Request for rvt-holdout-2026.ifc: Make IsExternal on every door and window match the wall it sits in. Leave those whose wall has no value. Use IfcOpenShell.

First a look at what the model holds.

```python
import ifcopenshell
import ifcopenshell.util.element

model = ifcopenshell.open("rvt-holdout-2026.ifc")
print(model.schema)
seen = {}
for e in model.by_type("IfcDoor") + model.by_type("IfcWindow"):
    if not e.FillsVoids:
        continue
    host = e.FillsVoids[0].RelatingOpeningElement.VoidsElements[0].RelatingBuildingElement
    own = ifcopenshell.util.element.get_pset(e, f"Pset_{e.is_a()[3:].removesuffix('StandardCase')}Common", "IsExternal")
    wall = ifcopenshell.util.element.get_pset(host, "Pset_WallCommon", "IsExternal")
    seen[e.is_a(), own, wall] = seen.get((e.is_a(), own, wall), 0) + 1
for (cls, own, wall), count in sorted(seen.items(), key=str):
    print(count, cls, "IsExternal:", own, "| host wall:", wall)
```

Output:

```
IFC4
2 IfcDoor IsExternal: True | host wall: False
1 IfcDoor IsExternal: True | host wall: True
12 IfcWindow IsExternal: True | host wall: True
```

```python
import ifcopenshell
import ifcopenshell.api.pset
import ifcopenshell.util.element

model = ifcopenshell.open("rvt-holdout-2026.ifc")

count = 0
for ifc_class, pset_name in (("IfcDoor", "Pset_DoorCommon"), ("IfcWindow", "Pset_WindowCommon")):
    for e in model.by_type(ifc_class):
        if not e.FillsVoids:
            continue
        host = e.FillsVoids[0].RelatingOpeningElement.VoidsElements[0].RelatingBuildingElement
        external = ifcopenshell.util.element.get_pset(host, "Pset_WallCommon", "IsExternal")
        if external is None or ifcopenshell.util.element.get_pset(e, pset_name, "IsExternal") == external:
            continue
        pset = ifcopenshell.api.pset.add_pset(model, product=e, name=pset_name)
        ifcopenshell.api.pset.edit_pset(model, pset=pset, properties={"IsExternal": external})
        count += 1

print(count, "updated")

model.write("rvt-holdout-2026_rev.ifc")
```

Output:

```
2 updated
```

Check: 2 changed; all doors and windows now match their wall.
